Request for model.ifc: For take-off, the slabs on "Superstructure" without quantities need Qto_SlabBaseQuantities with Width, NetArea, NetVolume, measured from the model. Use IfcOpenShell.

First a look at what the model holds.

```python
import ifcopenshell
import ifcopenshell.util.element
import ifcopenshell.util.unit

model = ifcopenshell.open("model.ifc")
print(model.schema)
for unit_type in ("LENGTHUNIT", "AREAUNIT", "VOLUMEUNIT"):
    print(unit_type, ifcopenshell.util.unit.calculate_unit_scale(model, unit_type))
storey = next(s for s in model.by_type("IfcBuildingStorey") if s.Name == "Superstructure")
slabs = [e for e in ifcopenshell.util.element.get_decomposition(storey) if e.is_a("IfcSlab")]
for e in sorted(slabs, key=lambda e: e.id()):
    print(e.id(), e.is_a(), e.Name, list(ifcopenshell.util.element.get_psets(e, qtos_only=True)), sep=" | ")
```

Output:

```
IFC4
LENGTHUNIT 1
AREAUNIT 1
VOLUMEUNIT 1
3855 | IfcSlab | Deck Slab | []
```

```python
import ifcopenshell
import ifcopenshell.api.pset
import ifcopenshell.geom
import ifcopenshell.util.element
import ifcopenshell.util.shape
import ifcopenshell.util.unit

model = ifcopenshell.open("model.ifc")
unit_scale = ifcopenshell.util.unit.calculate_unit_scale(model)
area_scale = ifcopenshell.util.unit.calculate_unit_scale(model, "AREAUNIT")
volume_scale = ifcopenshell.util.unit.calculate_unit_scale(model, "VOLUMEUNIT")
settings = ifcopenshell.geom.settings()

storey = next(s for s in model.by_type("IfcBuildingStorey") if s.Name == "Superstructure")
slabs = [e for e in ifcopenshell.util.element.get_decomposition(storey) if e.is_a("IfcSlab")]

for e in sorted(slabs, key=lambda e: e.id()):
    if ifcopenshell.util.element.get_psets(e, qtos_only=True, should_inherit=False):
        continue
    # Geometry comes back in metres, in the element's own axes.
    shape = ifcopenshell.geom.create_shape(settings, e)
    values = {
        "Width": ifcopenshell.util.shape.get_z(shape.geometry) / unit_scale,
        "NetArea": ifcopenshell.util.shape.get_footprint_area(shape.geometry) / area_scale,
        "NetVolume": ifcopenshell.util.shape.get_volume(shape.geometry) / volume_scale,
    }
    qto = ifcopenshell.api.pset.add_qto(model, product=e, name="Qto_SlabBaseQuantities")
    ifcopenshell.api.pset.edit_qto(model, qto=qto, properties=values)
    print(e.id(), {k: round(v, 3) for k, v in values.items()})

model.write("model_rev.ifc")
```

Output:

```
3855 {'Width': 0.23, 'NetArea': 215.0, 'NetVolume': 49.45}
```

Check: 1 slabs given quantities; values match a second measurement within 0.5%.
